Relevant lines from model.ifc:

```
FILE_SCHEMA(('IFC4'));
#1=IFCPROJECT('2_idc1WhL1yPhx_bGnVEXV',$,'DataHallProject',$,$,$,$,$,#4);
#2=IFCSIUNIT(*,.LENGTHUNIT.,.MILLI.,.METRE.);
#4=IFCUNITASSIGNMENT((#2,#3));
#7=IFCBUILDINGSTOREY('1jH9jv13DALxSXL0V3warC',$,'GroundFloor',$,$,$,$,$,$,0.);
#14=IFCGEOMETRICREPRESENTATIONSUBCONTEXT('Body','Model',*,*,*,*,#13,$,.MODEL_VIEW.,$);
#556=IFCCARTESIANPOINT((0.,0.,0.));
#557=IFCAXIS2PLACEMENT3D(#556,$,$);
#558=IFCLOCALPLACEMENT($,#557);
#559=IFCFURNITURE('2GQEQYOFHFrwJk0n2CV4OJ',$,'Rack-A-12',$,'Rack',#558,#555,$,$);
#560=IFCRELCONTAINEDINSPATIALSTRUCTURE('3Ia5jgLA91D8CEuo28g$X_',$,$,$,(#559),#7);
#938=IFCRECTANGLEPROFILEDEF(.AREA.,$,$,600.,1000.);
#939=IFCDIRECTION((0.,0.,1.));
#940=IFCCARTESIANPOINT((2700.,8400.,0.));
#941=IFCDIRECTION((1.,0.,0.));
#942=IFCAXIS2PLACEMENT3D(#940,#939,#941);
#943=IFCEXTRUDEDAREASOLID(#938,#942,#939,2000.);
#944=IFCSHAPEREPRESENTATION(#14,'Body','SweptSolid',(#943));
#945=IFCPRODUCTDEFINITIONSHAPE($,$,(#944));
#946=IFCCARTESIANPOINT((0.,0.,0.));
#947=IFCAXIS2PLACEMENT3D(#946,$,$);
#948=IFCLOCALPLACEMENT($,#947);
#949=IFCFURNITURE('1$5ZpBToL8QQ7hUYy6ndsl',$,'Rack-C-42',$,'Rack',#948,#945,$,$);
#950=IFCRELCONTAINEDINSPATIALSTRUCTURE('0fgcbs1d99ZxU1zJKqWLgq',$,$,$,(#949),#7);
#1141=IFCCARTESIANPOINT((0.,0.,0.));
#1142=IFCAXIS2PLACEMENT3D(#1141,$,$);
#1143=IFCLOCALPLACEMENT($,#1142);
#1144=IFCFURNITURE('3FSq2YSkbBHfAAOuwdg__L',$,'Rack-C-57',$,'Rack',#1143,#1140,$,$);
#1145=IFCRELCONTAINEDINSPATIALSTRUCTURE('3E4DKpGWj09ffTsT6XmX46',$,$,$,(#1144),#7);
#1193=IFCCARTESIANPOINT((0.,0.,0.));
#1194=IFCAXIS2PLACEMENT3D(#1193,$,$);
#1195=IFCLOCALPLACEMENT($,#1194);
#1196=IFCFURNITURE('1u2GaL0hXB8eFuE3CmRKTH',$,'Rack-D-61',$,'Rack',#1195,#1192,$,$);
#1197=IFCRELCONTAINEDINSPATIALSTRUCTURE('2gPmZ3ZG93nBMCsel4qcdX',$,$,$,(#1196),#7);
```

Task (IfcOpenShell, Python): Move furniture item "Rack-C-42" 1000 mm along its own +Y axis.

```python
import ifcopenshell
import ifcopenshell.api.geometry
import ifcopenshell.util.placement
import ifcopenshell.util.unit

model = ifcopenshell.open("model.ifc")
unit_scale = ifcopenshell.util.unit.calculate_unit_scale(model)

item = model.by_guid("1$5ZpBToL8QQ7hUYy6ndsl")
matrix = ifcopenshell.util.placement.get_local_placement(item.ObjectPlacement)
matrix[:3, 3] += matrix[:3, 1] * 1 / unit_scale
ifcopenshell.api.geometry.edit_object_placement(model, product=item, matrix=matrix, is_si=False)

print(ifcopenshell.util.placement.get_local_placement(item.ObjectPlacement).round(3) + 0.0)

model.write("model_rev.ifc")
```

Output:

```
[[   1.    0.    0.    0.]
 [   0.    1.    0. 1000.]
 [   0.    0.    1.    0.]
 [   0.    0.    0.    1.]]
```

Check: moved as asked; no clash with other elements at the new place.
